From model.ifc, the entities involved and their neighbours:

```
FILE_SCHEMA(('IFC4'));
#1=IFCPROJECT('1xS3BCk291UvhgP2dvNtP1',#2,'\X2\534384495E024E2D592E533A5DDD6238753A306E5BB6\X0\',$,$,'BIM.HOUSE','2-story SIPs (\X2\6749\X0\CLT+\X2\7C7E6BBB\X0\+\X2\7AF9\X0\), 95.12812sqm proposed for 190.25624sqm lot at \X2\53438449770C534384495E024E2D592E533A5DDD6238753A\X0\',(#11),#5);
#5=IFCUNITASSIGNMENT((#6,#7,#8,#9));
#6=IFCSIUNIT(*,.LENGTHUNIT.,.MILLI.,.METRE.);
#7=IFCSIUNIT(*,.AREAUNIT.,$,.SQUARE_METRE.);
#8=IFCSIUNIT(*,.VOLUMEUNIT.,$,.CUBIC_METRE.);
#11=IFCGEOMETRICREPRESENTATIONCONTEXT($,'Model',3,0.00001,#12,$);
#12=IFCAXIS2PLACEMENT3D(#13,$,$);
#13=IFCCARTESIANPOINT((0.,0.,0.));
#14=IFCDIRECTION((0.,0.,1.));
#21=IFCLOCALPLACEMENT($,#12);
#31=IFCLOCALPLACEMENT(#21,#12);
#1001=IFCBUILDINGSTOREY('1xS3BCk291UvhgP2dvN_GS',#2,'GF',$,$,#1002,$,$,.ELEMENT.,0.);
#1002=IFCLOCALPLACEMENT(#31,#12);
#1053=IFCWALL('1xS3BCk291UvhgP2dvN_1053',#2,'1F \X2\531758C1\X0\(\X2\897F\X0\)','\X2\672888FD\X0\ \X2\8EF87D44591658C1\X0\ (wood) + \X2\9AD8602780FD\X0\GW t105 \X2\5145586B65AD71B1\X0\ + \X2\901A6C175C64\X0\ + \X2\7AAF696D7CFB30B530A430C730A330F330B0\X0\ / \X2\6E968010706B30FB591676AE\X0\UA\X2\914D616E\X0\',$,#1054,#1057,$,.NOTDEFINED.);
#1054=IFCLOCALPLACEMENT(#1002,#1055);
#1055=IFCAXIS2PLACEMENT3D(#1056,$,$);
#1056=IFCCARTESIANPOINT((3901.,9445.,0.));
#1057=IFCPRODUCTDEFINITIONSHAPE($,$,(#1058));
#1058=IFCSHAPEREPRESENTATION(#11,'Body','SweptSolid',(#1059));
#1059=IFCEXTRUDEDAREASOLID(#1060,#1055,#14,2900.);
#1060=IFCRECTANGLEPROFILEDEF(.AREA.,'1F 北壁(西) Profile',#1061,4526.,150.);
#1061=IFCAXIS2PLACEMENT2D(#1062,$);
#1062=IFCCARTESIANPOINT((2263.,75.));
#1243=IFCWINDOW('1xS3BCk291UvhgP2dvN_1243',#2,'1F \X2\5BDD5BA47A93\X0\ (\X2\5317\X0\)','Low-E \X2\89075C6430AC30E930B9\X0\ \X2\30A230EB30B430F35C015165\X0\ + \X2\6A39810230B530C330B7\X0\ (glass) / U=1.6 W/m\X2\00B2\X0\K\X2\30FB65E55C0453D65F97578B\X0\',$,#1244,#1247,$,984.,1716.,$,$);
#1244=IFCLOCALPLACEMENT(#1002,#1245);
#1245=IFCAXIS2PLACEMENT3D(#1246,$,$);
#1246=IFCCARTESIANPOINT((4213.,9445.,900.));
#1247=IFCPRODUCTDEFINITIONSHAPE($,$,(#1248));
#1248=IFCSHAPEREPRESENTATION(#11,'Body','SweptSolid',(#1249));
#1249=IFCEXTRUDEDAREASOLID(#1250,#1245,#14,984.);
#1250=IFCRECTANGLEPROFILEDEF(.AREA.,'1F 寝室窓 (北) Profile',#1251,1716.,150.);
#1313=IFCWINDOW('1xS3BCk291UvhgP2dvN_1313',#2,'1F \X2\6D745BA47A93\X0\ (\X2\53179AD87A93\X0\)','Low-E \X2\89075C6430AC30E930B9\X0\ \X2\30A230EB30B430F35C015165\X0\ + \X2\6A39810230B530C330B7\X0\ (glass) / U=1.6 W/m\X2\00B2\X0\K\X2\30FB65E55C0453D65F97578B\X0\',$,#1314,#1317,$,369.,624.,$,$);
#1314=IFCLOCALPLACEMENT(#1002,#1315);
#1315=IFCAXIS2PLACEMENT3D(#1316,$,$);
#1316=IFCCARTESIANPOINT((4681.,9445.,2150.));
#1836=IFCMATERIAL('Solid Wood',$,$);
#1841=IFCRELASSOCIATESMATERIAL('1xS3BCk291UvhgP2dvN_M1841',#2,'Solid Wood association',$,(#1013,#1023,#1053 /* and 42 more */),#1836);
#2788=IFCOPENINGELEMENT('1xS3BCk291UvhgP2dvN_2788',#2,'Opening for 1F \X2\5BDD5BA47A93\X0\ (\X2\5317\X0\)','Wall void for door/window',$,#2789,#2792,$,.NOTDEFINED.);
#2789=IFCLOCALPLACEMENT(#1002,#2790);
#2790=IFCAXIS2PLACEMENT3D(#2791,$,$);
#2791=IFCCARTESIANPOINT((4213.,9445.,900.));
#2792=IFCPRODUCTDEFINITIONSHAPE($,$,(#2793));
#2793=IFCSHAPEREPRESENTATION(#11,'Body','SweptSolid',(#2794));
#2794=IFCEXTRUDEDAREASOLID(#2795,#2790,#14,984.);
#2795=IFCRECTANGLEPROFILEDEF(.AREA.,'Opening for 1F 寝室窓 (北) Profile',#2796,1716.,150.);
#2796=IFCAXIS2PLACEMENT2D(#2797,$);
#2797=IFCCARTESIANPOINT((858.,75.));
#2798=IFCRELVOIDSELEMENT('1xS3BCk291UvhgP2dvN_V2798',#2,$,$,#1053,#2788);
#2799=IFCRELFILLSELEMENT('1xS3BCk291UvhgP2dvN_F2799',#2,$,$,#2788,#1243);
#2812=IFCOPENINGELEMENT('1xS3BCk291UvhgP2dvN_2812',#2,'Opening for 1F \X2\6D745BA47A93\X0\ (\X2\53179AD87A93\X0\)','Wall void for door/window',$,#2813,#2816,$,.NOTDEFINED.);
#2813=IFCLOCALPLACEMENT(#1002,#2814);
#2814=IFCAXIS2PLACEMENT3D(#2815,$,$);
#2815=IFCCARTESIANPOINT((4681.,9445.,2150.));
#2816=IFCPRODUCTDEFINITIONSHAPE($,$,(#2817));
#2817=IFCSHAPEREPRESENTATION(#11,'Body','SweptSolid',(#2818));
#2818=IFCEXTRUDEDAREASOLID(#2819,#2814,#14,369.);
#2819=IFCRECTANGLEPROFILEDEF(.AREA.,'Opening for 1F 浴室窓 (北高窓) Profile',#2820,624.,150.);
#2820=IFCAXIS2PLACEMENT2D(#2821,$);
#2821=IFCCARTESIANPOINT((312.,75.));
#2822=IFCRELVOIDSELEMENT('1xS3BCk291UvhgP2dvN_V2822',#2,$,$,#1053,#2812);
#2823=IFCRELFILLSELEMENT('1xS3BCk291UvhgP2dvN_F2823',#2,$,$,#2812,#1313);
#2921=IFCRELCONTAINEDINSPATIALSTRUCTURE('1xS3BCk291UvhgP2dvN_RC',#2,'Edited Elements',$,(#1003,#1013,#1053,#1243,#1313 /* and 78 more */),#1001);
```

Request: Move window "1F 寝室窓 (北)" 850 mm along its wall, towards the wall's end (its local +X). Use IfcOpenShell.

```python
import ifcopenshell
import ifcopenshell.api.geometry
import ifcopenshell.util.placement
import ifcopenshell.util.unit

model = ifcopenshell.open("model.ifc")
unit_scale = ifcopenshell.util.unit.calculate_unit_scale(model)

window = model.by_guid("1xS3BCk291UvhgP2dvN_1243")
opening = window.FillsVoids[0].RelatingOpeningElement
wall = opening.VoidsElements[0].RelatingBuildingElement

wall_matrix = ifcopenshell.util.placement.get_local_placement(wall.ObjectPlacement)
shift = wall_matrix[:3, 0] * 0.85 / unit_scale
before = ifcopenshell.util.placement.get_local_placement(window.ObjectPlacement)[:3, 3].copy()

# The window is not placed relative to its opening, so move both.
for product in (opening, window):
    matrix = ifcopenshell.util.placement.get_local_placement(product.ObjectPlacement)
    matrix[:3, 3] += shift
    ifcopenshell.api.geometry.edit_object_placement(model, product=product, matrix=matrix, is_si=False)

after = ifcopenshell.util.placement.get_local_placement(window.ObjectPlacement)[:3, 3]
print("window moved by", (after - before).round(3) + 0.0)

model.write("model-out.ifc")
```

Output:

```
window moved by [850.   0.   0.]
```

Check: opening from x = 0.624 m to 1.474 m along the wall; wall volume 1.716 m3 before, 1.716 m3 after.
